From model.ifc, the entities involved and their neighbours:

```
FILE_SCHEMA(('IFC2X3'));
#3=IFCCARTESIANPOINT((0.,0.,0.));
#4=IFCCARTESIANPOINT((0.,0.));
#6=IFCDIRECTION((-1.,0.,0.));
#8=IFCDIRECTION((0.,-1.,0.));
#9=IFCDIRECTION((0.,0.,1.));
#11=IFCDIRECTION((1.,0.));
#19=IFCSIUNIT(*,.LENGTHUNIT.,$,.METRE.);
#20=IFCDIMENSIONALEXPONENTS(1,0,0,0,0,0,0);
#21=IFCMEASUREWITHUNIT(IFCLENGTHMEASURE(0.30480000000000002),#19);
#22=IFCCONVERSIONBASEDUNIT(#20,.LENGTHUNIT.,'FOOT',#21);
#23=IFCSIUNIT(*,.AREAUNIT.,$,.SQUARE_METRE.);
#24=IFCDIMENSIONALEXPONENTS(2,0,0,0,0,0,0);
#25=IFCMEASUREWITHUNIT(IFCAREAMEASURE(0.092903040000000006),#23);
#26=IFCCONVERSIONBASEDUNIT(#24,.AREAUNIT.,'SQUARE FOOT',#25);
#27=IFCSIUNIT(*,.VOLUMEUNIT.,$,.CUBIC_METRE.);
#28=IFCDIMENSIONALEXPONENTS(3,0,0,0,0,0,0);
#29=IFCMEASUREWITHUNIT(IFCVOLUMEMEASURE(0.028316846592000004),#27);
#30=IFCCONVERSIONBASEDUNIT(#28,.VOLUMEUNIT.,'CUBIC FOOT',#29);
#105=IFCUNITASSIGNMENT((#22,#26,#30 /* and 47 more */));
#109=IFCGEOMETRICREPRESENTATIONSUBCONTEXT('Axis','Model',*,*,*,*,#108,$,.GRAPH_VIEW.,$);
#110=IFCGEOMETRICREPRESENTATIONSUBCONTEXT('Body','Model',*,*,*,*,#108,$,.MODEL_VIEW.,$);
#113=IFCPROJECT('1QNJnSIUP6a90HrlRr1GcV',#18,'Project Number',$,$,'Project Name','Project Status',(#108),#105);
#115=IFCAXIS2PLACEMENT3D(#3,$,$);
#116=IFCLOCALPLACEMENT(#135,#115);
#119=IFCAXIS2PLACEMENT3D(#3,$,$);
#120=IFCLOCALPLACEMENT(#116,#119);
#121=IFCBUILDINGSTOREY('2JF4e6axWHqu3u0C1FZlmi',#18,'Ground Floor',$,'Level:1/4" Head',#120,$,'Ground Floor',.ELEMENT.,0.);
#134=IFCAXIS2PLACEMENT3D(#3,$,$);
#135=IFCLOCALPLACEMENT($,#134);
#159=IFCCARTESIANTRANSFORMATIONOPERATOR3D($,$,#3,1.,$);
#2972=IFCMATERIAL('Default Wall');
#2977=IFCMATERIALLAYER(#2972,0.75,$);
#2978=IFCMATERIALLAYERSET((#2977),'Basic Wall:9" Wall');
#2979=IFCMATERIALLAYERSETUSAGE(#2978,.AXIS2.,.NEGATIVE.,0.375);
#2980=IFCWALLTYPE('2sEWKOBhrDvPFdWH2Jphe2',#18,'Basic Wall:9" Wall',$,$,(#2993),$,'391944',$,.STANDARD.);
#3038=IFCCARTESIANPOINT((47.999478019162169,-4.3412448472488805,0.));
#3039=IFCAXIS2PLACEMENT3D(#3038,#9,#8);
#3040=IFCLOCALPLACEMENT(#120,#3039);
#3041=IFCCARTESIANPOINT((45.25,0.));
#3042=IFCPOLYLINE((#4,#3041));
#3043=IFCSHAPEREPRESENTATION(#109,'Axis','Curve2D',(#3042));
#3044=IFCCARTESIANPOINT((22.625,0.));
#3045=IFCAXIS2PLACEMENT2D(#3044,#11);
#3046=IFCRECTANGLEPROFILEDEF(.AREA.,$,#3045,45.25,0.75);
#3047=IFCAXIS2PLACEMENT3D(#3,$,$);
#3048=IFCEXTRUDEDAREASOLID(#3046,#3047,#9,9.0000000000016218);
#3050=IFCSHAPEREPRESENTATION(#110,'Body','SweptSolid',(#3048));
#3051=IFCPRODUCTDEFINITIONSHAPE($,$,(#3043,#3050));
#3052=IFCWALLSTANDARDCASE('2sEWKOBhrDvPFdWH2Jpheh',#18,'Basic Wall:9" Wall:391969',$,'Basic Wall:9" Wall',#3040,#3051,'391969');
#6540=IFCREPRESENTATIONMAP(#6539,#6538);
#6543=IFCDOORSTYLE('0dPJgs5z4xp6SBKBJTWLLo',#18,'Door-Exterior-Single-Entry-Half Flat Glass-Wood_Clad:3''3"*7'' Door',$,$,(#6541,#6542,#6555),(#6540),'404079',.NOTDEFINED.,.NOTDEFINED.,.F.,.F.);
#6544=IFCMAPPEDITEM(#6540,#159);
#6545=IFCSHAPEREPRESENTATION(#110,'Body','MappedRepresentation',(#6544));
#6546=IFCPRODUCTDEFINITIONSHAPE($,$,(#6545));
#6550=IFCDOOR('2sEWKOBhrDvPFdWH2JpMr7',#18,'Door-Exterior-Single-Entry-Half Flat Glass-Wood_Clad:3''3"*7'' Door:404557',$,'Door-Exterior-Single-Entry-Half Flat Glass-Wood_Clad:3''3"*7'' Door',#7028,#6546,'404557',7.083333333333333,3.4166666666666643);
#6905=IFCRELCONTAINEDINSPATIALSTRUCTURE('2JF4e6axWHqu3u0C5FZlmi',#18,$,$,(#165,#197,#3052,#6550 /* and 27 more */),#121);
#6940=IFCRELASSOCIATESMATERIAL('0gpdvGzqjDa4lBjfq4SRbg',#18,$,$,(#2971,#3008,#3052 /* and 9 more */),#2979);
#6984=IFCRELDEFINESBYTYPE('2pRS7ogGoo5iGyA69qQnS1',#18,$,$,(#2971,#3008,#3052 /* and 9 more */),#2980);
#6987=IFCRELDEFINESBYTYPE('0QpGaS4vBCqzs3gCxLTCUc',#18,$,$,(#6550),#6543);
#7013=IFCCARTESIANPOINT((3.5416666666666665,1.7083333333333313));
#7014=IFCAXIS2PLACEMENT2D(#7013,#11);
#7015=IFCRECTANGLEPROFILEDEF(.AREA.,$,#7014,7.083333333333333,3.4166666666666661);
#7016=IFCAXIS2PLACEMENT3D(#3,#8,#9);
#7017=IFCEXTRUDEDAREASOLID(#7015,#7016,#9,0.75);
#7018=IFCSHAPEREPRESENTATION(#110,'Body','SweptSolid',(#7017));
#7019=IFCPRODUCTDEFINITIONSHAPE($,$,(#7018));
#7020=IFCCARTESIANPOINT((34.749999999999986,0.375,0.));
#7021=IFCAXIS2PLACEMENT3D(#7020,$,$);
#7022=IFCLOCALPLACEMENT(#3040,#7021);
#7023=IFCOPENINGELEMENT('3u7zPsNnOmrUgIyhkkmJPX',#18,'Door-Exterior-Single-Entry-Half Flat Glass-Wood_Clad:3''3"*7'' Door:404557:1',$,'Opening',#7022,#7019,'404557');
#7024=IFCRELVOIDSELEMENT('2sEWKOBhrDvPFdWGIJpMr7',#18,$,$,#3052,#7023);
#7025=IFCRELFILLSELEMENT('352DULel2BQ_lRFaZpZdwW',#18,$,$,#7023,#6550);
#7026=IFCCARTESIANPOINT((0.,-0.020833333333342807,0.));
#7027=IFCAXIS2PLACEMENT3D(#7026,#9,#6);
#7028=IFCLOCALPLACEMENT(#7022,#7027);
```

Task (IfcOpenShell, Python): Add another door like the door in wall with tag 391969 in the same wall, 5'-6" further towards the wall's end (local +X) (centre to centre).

```python
import ifcopenshell
import ifcopenshell.api.feature
import ifcopenshell.api.geometry
import ifcopenshell.api.root
import ifcopenshell.geom
import ifcopenshell.util.element
import ifcopenshell.util.placement
import ifcopenshell.util.shape
import ifcopenshell.util.unit

model = ifcopenshell.open("model.ifc")
unit_scale = ifcopenshell.util.unit.calculate_unit_scale(model)
settings = ifcopenshell.geom.settings()


def volume(element):
    """Net volume in cubic metres, openings subtracted."""
    shape = ifcopenshell.geom.create_shape(settings, element)
    return ifcopenshell.util.shape.get_volume(shape.geometry)


def reuse_history(source, copy):
    """copy_class also copies each property set's owner history, people and application; keep the originals."""
    for rel in copy.IsDefinedBy:
        if rel.is_a("IfcRelDefinesByProperties") and (history := rel.RelatingPropertyDefinition.OwnerHistory):
            rel.RelatingPropertyDefinition.OwnerHistory = source.OwnerHistory
            ifcopenshell.util.element.remove_deep2(model, history)


door = model.by_guid("2sEWKOBhrDvPFdWH2JpMr7")
opening = door.FillsVoids[0].RelatingOpeningElement
wall = opening.VoidsElements[0].RelatingBuildingElement
before = volume(wall)
shift = ifcopenshell.util.placement.get_local_placement(wall.ObjectPlacement)[:3, 0] * 66 * 0.0254 / unit_scale

# copy_class copies the void relationship, type, container and properties, but no geometry.
new_opening = ifcopenshell.api.root.copy_class(model, product=opening)
new_opening.Representation = ifcopenshell.util.element.copy_deep(
    model, opening.Representation, exclude=["IfcGeometricRepresentationContext", "IfcRepresentationMap"]
)
new_opening.Name = 'Door-Exterior-Single-Entry-Half Flat Glass-Wood_Clad:3\'3"*7\' Door'
new_opening.Tag = None
new_door = ifcopenshell.api.root.copy_class(model, product=door)
new_door.Representation = ifcopenshell.util.element.copy_deep(
    model, door.Representation, exclude=["IfcGeometricRepresentationContext", "IfcRepresentationMap"]
)
new_door.Name = 'Door-Exterior-Single-Entry-Half Flat Glass-Wood_Clad:3\'3"*7\' Door'
new_door.Tag = None
reuse_history(door, new_door)
fills = ifcopenshell.api.feature.add_filling(model, opening=new_opening, element=new_door)
fills.OwnerHistory = new_door.OwnerHistory  # required in IFC2X3

for old, new in ((opening, new_opening), (door, new_door)):
    matrix = ifcopenshell.util.placement.get_local_placement(old.ObjectPlacement)
    matrix[:3, 3] += shift
    ifcopenshell.api.geometry.edit_object_placement(model, product=new, matrix=matrix, is_si=False)

after = volume(wall)

print(f"wall volume {before:.3f} -> {after:.3f} m3")

model.write("model_edited.ifc")
```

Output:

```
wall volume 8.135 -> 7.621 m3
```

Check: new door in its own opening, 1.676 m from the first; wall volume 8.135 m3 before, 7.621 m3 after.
